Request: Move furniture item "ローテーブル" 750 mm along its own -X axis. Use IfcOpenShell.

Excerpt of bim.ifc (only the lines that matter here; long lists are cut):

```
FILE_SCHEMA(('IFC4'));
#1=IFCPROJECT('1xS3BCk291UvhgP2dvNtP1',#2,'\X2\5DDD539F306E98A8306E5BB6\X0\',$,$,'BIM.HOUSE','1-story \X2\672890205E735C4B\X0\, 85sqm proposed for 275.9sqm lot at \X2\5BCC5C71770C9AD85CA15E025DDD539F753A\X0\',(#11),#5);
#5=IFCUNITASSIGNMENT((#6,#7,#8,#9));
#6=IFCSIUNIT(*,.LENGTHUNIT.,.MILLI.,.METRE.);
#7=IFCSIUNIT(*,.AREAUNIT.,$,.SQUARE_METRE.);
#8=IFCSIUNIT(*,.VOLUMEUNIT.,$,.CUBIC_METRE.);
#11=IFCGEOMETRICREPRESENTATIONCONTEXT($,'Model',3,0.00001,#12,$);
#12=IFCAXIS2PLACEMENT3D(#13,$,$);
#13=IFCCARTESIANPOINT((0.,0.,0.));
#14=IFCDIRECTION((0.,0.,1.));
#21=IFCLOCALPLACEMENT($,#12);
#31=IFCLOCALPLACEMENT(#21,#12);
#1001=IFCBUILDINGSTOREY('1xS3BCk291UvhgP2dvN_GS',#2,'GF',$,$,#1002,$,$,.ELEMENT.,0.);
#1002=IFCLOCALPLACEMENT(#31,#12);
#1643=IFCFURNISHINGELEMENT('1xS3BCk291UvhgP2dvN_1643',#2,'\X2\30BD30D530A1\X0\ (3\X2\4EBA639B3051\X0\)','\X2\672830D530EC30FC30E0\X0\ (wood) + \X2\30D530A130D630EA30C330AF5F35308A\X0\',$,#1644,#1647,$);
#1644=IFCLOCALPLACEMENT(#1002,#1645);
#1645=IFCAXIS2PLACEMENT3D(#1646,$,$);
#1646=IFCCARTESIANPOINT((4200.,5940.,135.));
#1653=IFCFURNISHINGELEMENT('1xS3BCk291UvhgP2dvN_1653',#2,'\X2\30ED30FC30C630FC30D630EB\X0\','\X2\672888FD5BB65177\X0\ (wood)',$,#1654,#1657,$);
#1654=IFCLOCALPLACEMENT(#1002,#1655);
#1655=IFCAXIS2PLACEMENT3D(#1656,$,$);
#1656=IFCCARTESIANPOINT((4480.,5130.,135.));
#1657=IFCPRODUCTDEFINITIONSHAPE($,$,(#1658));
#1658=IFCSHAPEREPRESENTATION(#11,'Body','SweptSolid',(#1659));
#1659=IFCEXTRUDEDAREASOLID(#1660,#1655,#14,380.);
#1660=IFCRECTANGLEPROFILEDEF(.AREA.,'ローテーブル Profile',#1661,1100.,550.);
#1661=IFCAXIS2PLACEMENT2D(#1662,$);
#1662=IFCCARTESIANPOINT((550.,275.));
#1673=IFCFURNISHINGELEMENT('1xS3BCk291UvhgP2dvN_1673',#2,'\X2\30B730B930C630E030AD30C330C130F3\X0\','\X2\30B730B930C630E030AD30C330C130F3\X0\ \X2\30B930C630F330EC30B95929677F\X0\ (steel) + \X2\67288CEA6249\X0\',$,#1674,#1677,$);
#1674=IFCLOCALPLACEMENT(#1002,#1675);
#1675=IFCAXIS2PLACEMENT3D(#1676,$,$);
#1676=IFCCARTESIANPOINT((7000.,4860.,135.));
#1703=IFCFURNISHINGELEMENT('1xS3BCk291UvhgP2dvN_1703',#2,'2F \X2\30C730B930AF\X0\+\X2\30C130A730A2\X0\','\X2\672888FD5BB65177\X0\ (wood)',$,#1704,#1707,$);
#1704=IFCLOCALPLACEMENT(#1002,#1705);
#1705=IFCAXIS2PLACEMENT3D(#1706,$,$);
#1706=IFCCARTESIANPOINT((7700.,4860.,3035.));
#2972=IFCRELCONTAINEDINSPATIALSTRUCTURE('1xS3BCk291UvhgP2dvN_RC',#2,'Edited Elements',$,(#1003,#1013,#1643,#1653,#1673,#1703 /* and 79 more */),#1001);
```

```python
import ifcopenshell
import ifcopenshell.api.geometry
import ifcopenshell.util.placement
import ifcopenshell.util.unit

model = ifcopenshell.open("bim.ifc")
unit_scale = ifcopenshell.util.unit.calculate_unit_scale(model)

item = model.by_guid("1xS3BCk291UvhgP2dvN_1653")
matrix = ifcopenshell.util.placement.get_local_placement(item.ObjectPlacement)
matrix[:3, 3] -= matrix[:3, 0] * 0.75 / unit_scale
ifcopenshell.api.geometry.edit_object_placement(model, product=item, matrix=matrix, is_si=False)

print(ifcopenshell.util.placement.get_local_placement(item.ObjectPlacement).round(3) + 0.0)

model.write("bim-out.ifc")
```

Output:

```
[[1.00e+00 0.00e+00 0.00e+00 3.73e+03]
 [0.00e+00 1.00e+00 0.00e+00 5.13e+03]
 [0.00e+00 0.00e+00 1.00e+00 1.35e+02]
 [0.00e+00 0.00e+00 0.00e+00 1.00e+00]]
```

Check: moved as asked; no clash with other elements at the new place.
